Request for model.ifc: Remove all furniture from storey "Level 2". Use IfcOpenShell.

First a look at what the model holds.

```python
import ifcopenshell
import ifcopenshell.util.element

model = ifcopenshell.open("model.ifc")
print(model.schema)
storey = next(s for s in model.by_type("IfcBuildingStorey") if s.Name == "Level 2")
furniture = [e for e in ifcopenshell.util.element.get_decomposition(storey) if e.is_a("IfcFurnishingElement")]
seen = {}
for e in furniture:
    element_type = ifcopenshell.util.element.get_type(e)
    name = element_type.Name if element_type not in (None, e) else None
    seen[name] = seen.get(name, 0) + 1
for name, count in sorted(seen.items(), key=str):
    print(count, "x", name)
```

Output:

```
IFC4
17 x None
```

```python
import ifcopenshell
import ifcopenshell.api.root
import ifcopenshell.util.element

model = ifcopenshell.open("model.ifc")

storey = next(s for s in model.by_type("IfcBuildingStorey") if s.Name == "Level 2")
furniture = [e for e in ifcopenshell.util.element.get_decomposition(storey) if e.is_a("IfcFurnishingElement")]

for e in furniture:
    ifcopenshell.api.root.remove_product(model, product=e)
print(len(furniture), "removed")

model.write("model_v2.ifc")
```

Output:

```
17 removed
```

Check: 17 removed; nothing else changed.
